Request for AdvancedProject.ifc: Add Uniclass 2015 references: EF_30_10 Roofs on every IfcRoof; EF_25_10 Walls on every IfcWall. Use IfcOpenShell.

First a look at what the model holds.

```python
import ifcopenshell

model = ifcopenshell.open("AdvancedProject.ifc")
print(model.schema)
print("classifications:", [c.Name for c in model.by_type("IfcClassification")])
for ifc_class in ("IfcDoor", "IfcRoof", "IfcStair", "IfcWall", "IfcWindow"):
    print(ifc_class, len(model.by_type(ifc_class)))
```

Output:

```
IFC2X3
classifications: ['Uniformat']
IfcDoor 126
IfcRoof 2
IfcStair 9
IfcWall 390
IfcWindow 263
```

```python
import ifcopenshell
import ifcopenshell.api.classification

model = ifcopenshell.open("AdvancedProject.ifc")

# IFC2X3 requires Source and Edition and has no link from the project to the system.
system = model.create_entity("IfcClassification", Source="NBS", Edition="2015", Name="Uniclass 2015")

codes = {
    "IfcRoof": ("EF_30_10", "Roofs"),
    "IfcWall": ("EF_25_10", "Walls"),
}
for ifc_class, (code, name) in codes.items():
    products = model.by_type(ifc_class)
    ifcopenshell.api.classification.add_reference(
        model, products=products, classification=system, identification=code, name=name
    )
    print(code, len(products))

model.write("AdvancedProject-out.ifc")
```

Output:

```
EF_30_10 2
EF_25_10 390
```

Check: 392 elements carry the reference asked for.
